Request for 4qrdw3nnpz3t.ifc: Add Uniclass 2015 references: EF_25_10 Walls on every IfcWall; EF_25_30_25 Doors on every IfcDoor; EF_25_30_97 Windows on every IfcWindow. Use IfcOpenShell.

First a look at what the model holds.

```python
import ifcopenshell

model = ifcopenshell.open("4qrdw3nnpz3t.ifc")
print(model.schema)
print("classifications:", [c.Name for c in model.by_type("IfcClassification")])
for ifc_class in ("IfcDoor", "IfcRoof", "IfcStair", "IfcWall", "IfcWindow"):
    print(ifc_class, len(model.by_type(ifc_class)))
```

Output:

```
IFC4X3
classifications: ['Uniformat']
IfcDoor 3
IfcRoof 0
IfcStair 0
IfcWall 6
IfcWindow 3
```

```python
import ifcopenshell
import ifcopenshell.api.classification

model = ifcopenshell.open("4qrdw3nnpz3t.ifc")

system = ifcopenshell.api.classification.add_classification(model, classification="Uniclass 2015")

codes = {
    "IfcWall": ("EF_25_10", "Walls"),
    "IfcDoor": ("EF_25_30_25", "Doors"),
    "IfcWindow": ("EF_25_30_97", "Windows"),
}
for ifc_class, (code, name) in codes.items():
    products = model.by_type(ifc_class)
    ifcopenshell.api.classification.add_reference(
        model, products=products, classification=system, identification=code, name=name
    )
    print(code, len(products))

model.write("4qrdw3nnpz3t_v2.ifc")
```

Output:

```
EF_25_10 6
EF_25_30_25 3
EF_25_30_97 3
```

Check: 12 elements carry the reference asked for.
